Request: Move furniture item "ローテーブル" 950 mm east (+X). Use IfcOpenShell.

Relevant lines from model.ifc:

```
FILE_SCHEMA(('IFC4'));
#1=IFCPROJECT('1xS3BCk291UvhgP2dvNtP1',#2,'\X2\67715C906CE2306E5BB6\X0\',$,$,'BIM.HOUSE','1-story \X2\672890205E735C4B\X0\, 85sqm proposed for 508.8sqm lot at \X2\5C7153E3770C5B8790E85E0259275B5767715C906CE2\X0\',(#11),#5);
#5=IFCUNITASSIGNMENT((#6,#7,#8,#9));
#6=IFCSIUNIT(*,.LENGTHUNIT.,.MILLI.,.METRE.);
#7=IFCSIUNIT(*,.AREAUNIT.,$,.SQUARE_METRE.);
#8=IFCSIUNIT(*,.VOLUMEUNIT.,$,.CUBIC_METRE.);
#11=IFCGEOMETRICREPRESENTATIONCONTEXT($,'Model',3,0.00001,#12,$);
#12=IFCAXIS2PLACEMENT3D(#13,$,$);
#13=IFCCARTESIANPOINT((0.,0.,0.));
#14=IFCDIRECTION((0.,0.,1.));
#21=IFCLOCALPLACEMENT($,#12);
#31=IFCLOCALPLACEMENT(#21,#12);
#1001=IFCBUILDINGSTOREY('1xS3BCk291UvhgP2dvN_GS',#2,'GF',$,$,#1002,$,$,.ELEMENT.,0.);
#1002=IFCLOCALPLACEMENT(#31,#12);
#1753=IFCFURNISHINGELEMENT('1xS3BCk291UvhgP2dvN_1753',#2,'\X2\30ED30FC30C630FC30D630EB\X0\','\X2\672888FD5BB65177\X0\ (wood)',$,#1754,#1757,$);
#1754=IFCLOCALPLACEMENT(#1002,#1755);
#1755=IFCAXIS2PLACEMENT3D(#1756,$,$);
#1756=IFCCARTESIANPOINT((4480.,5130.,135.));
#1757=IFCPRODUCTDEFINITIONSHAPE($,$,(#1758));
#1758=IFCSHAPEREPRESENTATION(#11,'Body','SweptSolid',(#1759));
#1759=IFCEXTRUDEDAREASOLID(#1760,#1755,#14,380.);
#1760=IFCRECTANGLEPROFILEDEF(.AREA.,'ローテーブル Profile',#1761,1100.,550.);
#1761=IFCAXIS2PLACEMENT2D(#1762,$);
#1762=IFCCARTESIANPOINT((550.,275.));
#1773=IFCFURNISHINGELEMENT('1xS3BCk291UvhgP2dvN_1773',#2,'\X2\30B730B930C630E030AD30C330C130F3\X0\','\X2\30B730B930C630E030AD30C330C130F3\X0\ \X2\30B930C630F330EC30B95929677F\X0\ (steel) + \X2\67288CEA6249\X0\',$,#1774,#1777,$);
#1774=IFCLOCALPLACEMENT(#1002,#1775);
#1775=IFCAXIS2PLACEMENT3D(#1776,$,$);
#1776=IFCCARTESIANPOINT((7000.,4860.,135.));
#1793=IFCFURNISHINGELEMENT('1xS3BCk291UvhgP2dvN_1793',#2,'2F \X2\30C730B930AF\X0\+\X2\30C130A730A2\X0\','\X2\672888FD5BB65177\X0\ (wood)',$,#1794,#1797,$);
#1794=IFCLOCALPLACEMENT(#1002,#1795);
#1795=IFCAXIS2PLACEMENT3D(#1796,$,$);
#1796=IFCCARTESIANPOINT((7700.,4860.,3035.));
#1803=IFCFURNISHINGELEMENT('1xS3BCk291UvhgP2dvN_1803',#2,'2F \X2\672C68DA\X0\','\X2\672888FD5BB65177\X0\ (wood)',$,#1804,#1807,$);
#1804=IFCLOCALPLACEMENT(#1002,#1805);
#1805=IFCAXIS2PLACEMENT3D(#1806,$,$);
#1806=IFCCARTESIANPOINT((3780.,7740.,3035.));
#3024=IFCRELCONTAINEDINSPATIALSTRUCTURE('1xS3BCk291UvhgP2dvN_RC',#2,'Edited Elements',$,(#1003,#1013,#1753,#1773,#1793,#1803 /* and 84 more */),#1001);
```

```python
import ifcopenshell
import ifcopenshell.api.geometry
import ifcopenshell.util.placement
import ifcopenshell.util.unit

model = ifcopenshell.open("model.ifc")
unit_scale = ifcopenshell.util.unit.calculate_unit_scale(model)

item = model.by_guid("1xS3BCk291UvhgP2dvN_1753")
matrix = ifcopenshell.util.placement.get_local_placement(item.ObjectPlacement)
matrix[0, 3] += 0.95 / unit_scale
ifcopenshell.api.geometry.edit_object_placement(model, product=item, matrix=matrix, is_si=False)

print(ifcopenshell.util.placement.get_local_placement(item.ObjectPlacement).round(3) + 0.0)

model.write("model_updated.ifc")
```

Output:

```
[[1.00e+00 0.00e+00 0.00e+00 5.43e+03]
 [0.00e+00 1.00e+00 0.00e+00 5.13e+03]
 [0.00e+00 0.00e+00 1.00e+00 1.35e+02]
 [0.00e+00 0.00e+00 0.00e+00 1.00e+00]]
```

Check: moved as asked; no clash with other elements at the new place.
